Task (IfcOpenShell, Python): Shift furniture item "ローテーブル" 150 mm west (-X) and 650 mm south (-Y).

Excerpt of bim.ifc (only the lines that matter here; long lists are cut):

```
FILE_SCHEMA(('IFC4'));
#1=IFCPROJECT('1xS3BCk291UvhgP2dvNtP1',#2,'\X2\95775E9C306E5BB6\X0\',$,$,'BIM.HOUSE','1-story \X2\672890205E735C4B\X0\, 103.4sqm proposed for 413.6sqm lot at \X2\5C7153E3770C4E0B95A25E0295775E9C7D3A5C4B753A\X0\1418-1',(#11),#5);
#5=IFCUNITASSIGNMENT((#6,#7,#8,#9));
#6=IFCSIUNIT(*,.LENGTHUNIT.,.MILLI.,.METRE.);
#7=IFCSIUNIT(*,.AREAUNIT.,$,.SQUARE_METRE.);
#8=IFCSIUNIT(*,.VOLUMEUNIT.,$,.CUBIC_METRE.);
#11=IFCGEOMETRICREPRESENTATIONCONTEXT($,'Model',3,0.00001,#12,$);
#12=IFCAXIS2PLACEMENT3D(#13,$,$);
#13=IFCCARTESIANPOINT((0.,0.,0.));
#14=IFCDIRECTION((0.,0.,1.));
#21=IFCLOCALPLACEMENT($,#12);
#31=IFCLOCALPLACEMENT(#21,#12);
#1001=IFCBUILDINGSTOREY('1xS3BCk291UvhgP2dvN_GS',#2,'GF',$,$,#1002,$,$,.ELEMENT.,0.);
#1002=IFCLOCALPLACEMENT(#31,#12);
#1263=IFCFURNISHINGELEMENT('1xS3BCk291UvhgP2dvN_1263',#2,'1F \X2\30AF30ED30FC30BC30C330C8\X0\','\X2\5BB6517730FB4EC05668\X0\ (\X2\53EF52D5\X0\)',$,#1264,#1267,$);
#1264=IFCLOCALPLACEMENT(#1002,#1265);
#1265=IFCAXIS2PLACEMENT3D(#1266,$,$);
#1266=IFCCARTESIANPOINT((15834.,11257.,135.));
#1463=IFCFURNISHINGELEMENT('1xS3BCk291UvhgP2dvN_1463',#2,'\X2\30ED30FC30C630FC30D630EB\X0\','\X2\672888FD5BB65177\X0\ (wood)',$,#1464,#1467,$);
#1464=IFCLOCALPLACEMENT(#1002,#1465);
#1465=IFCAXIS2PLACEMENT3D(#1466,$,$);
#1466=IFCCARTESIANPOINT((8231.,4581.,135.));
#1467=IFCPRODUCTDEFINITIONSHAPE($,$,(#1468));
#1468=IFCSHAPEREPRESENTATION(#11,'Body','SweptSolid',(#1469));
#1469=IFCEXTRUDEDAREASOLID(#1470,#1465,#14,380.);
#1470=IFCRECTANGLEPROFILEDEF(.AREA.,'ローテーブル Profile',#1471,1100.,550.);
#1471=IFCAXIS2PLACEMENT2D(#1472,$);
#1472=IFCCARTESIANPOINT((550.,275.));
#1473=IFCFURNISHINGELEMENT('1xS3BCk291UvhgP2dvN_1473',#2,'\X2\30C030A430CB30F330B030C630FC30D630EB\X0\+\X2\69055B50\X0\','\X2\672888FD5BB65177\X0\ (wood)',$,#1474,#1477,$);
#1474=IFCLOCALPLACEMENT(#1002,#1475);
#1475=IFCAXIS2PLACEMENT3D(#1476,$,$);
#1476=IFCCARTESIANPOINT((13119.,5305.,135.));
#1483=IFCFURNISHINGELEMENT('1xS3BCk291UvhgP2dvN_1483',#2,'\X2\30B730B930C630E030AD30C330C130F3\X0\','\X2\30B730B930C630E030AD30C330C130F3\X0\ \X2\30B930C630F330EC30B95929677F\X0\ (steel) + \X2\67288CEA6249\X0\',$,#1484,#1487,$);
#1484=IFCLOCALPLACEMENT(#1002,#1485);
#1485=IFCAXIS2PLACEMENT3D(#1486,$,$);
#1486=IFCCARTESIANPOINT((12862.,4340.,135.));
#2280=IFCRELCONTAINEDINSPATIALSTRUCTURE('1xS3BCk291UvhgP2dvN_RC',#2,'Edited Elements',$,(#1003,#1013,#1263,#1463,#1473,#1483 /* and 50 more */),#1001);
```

```python
import ifcopenshell
import ifcopenshell.api.geometry
import ifcopenshell.util.placement

model = ifcopenshell.open("bim.ifc")

item = model.by_guid("1xS3BCk291UvhgP2dvN_1463")
matrix = ifcopenshell.util.placement.get_local_placement(item.ObjectPlacement)
matrix[0, 3] -= 150.0
matrix[1, 3] -= 650.0
ifcopenshell.api.geometry.edit_object_placement(model, product=item, matrix=matrix, is_si=False)

print(ifcopenshell.util.placement.get_local_placement(item.ObjectPlacement).round(3) + 0.0)

model.write("bim_rev.ifc")
```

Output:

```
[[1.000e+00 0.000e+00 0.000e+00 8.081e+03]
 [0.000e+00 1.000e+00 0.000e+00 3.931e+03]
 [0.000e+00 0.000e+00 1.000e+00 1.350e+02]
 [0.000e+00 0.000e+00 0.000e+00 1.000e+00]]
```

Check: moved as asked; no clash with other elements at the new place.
